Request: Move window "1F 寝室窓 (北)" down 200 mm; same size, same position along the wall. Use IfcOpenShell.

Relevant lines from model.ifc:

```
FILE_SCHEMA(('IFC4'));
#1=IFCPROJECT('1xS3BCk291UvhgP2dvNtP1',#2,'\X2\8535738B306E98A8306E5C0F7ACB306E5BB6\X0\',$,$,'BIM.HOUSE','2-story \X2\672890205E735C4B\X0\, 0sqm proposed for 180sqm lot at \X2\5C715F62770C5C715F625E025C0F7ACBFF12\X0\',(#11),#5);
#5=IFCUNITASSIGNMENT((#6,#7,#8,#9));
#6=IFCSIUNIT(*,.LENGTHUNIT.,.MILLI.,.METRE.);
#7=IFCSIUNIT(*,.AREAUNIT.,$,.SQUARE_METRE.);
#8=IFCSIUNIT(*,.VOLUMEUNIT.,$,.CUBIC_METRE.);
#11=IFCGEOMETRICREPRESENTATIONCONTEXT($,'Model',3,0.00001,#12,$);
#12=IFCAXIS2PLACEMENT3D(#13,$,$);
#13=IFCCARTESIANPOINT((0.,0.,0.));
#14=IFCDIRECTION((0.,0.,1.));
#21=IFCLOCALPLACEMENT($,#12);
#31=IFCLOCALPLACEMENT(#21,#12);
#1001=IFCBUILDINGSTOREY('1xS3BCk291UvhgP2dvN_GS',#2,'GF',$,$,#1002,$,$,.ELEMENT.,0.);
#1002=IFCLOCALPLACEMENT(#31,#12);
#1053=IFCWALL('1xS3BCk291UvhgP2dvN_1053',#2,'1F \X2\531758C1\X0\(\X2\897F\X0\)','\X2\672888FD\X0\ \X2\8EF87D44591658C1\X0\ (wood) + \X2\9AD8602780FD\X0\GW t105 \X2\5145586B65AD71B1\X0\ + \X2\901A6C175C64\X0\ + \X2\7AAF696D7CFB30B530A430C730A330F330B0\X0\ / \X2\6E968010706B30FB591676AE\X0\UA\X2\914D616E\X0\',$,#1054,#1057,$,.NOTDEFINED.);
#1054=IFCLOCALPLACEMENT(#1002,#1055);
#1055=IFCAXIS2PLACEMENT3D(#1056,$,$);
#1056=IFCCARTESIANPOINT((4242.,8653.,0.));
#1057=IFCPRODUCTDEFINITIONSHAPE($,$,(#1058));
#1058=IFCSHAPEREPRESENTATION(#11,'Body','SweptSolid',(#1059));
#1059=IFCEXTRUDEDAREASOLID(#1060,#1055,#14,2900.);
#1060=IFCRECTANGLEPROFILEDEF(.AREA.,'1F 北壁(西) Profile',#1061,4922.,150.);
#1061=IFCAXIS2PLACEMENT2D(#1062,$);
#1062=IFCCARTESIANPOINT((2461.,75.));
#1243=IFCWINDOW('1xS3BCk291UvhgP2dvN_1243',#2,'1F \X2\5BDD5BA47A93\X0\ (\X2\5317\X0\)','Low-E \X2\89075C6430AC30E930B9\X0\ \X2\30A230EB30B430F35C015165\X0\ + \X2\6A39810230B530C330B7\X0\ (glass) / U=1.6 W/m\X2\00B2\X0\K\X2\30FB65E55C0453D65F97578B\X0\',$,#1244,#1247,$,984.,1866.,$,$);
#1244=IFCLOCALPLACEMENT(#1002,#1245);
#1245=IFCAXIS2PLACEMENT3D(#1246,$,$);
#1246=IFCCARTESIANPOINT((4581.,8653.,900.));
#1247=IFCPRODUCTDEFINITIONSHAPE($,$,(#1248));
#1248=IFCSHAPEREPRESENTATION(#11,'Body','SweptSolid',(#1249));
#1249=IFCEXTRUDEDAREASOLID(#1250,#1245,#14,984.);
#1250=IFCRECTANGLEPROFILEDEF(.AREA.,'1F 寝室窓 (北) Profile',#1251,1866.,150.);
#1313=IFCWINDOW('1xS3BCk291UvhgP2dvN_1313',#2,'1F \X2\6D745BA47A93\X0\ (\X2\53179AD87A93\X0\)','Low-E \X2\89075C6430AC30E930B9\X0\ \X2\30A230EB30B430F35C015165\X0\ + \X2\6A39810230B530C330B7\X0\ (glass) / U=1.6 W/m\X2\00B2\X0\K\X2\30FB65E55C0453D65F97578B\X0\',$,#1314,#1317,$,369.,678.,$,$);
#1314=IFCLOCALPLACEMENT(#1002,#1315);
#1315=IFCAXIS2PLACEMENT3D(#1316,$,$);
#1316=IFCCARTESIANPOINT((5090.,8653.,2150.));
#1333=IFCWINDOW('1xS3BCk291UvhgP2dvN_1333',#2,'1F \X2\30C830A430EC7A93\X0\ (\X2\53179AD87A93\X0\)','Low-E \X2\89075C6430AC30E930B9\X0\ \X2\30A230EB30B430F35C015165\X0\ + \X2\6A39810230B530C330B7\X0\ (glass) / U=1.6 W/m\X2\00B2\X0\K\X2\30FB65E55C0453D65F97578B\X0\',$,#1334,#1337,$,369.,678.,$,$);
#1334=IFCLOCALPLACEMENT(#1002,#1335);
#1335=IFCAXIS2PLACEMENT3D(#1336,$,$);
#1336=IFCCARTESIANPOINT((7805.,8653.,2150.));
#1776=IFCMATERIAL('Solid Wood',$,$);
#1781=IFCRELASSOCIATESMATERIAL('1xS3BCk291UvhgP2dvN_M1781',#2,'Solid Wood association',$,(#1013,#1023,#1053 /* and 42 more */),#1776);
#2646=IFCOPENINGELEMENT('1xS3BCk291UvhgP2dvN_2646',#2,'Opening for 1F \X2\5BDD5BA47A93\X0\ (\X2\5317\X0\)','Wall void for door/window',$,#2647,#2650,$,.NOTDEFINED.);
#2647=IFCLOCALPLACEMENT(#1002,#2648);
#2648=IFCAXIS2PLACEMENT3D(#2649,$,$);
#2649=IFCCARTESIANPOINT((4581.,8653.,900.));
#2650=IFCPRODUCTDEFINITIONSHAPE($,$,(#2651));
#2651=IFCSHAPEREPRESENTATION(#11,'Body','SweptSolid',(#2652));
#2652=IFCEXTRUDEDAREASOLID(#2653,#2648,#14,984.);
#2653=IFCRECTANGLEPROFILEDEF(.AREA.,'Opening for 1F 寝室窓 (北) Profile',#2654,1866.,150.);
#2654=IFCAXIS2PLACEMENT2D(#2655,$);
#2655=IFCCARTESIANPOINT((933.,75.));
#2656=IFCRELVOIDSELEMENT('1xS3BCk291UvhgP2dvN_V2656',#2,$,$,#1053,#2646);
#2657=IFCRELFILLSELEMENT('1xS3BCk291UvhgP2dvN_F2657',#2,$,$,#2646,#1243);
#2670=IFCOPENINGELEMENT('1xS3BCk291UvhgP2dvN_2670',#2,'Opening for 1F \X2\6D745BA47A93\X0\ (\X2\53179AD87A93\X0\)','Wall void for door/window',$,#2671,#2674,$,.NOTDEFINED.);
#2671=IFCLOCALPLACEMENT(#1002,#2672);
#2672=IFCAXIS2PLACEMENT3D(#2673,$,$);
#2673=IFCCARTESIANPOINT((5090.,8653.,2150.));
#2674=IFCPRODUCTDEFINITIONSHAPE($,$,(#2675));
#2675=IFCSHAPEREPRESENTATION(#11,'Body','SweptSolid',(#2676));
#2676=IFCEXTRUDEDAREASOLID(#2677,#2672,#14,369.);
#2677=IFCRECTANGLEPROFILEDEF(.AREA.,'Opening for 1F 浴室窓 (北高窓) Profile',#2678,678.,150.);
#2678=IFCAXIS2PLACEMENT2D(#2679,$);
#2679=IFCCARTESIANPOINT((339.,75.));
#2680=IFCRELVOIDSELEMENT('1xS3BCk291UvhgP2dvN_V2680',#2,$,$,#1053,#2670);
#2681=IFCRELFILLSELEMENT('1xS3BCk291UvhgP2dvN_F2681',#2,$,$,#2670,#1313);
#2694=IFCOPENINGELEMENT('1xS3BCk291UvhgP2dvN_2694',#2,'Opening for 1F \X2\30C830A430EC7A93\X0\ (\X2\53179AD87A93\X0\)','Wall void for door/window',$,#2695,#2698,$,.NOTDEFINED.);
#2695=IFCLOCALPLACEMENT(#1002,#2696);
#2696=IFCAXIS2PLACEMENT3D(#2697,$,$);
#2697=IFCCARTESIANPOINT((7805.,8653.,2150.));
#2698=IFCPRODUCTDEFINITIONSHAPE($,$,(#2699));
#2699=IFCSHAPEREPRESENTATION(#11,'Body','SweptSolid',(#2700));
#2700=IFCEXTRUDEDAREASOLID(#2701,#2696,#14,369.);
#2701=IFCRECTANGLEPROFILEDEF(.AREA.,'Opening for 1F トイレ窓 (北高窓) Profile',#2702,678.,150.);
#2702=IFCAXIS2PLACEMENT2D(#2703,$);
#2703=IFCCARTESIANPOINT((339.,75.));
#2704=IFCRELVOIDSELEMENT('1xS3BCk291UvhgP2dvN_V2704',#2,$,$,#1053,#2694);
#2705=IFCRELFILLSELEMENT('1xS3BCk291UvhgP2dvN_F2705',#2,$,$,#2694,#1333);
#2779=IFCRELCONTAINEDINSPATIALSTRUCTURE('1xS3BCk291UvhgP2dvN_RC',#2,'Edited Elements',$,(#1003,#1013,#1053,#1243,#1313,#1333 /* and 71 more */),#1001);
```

```python
import numpy as np
import ifcopenshell
import ifcopenshell.api.geometry
import ifcopenshell.util.placement
import ifcopenshell.util.unit

model = ifcopenshell.open("model.ifc")
unit_scale = ifcopenshell.util.unit.calculate_unit_scale(model)

window = model.by_id(1243)
opening = window.FillsVoids[0].RelatingOpeningElement
dz = -0.2 / unit_scale

shift = np.array([0.0, 0.0, dz])
# The window is not placed relative to its opening, so move both.
for product in (opening, window):
    matrix = ifcopenshell.util.placement.get_local_placement(product.ObjectPlacement)
    matrix[:3, 3] += shift
    ifcopenshell.api.geometry.edit_object_placement(model, product=product, matrix=matrix, is_si=False)

print(f"moved by {dz * unit_scale:+.3f} m")

model.write("model_rev.ifc")
```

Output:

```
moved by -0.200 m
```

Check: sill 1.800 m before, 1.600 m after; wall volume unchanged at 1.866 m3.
